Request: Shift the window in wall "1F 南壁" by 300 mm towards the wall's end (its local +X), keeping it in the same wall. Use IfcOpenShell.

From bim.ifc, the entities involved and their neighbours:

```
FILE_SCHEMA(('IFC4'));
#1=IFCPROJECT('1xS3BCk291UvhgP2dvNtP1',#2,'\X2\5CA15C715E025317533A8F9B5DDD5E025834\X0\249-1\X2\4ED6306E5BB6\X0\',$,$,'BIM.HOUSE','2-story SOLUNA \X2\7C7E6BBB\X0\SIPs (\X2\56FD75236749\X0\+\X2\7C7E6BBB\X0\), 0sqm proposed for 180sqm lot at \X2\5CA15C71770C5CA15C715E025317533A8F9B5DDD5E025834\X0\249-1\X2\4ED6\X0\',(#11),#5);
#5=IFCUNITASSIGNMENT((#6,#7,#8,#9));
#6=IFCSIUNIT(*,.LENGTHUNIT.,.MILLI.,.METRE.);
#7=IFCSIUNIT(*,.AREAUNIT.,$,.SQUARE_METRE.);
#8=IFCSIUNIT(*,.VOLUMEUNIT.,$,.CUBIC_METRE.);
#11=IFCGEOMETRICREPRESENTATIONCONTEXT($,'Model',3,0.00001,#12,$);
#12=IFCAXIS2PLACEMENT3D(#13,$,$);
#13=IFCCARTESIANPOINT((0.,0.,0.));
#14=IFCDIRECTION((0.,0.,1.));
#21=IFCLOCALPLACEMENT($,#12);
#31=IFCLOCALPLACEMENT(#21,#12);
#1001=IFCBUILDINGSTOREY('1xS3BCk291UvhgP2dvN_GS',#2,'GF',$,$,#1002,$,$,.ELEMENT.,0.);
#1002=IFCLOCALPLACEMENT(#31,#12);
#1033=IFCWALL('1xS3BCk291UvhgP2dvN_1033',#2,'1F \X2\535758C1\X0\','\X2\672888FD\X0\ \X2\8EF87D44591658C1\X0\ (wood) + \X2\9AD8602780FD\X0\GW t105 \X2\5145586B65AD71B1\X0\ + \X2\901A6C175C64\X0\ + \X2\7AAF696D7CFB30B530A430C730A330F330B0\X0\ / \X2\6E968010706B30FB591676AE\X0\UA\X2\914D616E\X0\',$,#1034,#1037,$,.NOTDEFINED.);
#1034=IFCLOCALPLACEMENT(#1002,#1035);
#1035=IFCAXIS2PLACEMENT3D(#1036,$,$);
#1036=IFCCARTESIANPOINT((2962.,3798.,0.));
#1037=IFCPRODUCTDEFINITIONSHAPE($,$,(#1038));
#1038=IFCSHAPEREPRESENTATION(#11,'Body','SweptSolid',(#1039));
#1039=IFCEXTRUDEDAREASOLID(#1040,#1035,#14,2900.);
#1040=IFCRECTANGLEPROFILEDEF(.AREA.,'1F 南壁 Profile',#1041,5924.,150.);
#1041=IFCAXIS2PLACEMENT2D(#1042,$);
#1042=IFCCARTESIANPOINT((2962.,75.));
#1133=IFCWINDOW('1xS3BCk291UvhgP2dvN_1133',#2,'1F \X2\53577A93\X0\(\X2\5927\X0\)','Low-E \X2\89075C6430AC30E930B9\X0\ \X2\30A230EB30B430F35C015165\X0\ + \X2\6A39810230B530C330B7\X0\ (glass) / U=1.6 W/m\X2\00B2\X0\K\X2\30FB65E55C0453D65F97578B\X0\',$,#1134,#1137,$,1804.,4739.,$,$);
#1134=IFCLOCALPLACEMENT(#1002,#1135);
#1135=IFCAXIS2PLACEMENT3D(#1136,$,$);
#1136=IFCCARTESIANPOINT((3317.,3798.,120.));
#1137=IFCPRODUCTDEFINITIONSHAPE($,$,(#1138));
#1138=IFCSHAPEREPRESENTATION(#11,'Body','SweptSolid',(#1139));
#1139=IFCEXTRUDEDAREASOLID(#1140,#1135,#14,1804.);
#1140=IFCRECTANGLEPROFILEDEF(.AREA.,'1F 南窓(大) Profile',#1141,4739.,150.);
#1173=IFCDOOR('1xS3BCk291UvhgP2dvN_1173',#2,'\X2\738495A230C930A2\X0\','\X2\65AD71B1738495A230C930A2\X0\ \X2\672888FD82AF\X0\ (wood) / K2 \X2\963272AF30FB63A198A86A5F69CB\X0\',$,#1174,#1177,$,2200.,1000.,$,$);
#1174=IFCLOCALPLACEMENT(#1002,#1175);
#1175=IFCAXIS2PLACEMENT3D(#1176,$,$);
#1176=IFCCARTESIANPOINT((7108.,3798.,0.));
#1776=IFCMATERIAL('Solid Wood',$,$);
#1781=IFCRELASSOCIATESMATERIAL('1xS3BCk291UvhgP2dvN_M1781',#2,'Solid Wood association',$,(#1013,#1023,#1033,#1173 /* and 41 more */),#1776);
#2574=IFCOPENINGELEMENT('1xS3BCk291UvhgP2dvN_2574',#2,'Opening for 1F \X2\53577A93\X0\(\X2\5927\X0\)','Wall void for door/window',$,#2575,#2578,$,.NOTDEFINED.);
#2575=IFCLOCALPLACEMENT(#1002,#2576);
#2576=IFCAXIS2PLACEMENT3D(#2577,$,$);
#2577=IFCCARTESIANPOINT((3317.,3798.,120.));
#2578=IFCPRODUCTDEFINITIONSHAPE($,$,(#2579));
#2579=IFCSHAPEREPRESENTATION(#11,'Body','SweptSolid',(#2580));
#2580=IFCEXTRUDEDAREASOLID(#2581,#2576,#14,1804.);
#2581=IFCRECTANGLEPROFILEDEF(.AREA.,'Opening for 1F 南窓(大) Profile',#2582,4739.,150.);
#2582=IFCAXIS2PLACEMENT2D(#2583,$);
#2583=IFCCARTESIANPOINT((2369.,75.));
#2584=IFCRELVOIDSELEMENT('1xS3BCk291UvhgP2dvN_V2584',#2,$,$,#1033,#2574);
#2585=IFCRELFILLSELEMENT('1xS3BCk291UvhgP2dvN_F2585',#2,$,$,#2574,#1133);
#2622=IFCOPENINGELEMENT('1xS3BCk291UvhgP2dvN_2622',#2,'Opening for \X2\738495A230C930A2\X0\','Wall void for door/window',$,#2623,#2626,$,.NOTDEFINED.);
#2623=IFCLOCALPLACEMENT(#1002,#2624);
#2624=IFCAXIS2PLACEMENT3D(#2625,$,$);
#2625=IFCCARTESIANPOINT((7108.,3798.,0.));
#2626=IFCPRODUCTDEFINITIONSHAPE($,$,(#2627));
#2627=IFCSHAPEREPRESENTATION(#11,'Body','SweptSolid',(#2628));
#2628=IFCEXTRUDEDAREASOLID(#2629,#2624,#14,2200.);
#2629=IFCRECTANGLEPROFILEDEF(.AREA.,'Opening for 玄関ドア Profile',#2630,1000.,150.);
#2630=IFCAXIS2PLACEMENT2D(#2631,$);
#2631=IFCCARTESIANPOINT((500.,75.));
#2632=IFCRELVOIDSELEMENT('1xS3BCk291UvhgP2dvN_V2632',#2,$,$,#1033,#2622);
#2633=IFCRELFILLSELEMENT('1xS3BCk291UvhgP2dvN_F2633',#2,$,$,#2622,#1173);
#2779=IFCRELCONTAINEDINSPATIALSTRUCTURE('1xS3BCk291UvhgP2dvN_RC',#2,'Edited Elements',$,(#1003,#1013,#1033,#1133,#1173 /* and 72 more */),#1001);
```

```python
import ifcopenshell
import ifcopenshell.api.geometry
import ifcopenshell.util.placement
import ifcopenshell.util.unit

model = ifcopenshell.open("bim.ifc")
unit_scale = ifcopenshell.util.unit.calculate_unit_scale(model)

window = model.by_id(1133)
opening = window.FillsVoids[0].RelatingOpeningElement
wall = opening.VoidsElements[0].RelatingBuildingElement

wall_matrix = ifcopenshell.util.placement.get_local_placement(wall.ObjectPlacement)
shift = wall_matrix[:3, 0] * 0.3 / unit_scale
before = ifcopenshell.util.placement.get_local_placement(window.ObjectPlacement)[:3, 3].copy()

# The window is not placed relative to its opening, so move both.
for product in (opening, window):
    matrix = ifcopenshell.util.placement.get_local_placement(product.ObjectPlacement)
    matrix[:3, 3] += shift
    ifcopenshell.api.geometry.edit_object_placement(model, product=product, matrix=matrix, is_si=False)

after = ifcopenshell.util.placement.get_local_placement(window.ObjectPlacement)[:3, 3]
print("window moved by", (after - before).round(3) + 0.0)

model.write("bim_v2.ifc")
```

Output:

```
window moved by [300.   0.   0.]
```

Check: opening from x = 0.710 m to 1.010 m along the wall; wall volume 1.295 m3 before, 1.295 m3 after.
